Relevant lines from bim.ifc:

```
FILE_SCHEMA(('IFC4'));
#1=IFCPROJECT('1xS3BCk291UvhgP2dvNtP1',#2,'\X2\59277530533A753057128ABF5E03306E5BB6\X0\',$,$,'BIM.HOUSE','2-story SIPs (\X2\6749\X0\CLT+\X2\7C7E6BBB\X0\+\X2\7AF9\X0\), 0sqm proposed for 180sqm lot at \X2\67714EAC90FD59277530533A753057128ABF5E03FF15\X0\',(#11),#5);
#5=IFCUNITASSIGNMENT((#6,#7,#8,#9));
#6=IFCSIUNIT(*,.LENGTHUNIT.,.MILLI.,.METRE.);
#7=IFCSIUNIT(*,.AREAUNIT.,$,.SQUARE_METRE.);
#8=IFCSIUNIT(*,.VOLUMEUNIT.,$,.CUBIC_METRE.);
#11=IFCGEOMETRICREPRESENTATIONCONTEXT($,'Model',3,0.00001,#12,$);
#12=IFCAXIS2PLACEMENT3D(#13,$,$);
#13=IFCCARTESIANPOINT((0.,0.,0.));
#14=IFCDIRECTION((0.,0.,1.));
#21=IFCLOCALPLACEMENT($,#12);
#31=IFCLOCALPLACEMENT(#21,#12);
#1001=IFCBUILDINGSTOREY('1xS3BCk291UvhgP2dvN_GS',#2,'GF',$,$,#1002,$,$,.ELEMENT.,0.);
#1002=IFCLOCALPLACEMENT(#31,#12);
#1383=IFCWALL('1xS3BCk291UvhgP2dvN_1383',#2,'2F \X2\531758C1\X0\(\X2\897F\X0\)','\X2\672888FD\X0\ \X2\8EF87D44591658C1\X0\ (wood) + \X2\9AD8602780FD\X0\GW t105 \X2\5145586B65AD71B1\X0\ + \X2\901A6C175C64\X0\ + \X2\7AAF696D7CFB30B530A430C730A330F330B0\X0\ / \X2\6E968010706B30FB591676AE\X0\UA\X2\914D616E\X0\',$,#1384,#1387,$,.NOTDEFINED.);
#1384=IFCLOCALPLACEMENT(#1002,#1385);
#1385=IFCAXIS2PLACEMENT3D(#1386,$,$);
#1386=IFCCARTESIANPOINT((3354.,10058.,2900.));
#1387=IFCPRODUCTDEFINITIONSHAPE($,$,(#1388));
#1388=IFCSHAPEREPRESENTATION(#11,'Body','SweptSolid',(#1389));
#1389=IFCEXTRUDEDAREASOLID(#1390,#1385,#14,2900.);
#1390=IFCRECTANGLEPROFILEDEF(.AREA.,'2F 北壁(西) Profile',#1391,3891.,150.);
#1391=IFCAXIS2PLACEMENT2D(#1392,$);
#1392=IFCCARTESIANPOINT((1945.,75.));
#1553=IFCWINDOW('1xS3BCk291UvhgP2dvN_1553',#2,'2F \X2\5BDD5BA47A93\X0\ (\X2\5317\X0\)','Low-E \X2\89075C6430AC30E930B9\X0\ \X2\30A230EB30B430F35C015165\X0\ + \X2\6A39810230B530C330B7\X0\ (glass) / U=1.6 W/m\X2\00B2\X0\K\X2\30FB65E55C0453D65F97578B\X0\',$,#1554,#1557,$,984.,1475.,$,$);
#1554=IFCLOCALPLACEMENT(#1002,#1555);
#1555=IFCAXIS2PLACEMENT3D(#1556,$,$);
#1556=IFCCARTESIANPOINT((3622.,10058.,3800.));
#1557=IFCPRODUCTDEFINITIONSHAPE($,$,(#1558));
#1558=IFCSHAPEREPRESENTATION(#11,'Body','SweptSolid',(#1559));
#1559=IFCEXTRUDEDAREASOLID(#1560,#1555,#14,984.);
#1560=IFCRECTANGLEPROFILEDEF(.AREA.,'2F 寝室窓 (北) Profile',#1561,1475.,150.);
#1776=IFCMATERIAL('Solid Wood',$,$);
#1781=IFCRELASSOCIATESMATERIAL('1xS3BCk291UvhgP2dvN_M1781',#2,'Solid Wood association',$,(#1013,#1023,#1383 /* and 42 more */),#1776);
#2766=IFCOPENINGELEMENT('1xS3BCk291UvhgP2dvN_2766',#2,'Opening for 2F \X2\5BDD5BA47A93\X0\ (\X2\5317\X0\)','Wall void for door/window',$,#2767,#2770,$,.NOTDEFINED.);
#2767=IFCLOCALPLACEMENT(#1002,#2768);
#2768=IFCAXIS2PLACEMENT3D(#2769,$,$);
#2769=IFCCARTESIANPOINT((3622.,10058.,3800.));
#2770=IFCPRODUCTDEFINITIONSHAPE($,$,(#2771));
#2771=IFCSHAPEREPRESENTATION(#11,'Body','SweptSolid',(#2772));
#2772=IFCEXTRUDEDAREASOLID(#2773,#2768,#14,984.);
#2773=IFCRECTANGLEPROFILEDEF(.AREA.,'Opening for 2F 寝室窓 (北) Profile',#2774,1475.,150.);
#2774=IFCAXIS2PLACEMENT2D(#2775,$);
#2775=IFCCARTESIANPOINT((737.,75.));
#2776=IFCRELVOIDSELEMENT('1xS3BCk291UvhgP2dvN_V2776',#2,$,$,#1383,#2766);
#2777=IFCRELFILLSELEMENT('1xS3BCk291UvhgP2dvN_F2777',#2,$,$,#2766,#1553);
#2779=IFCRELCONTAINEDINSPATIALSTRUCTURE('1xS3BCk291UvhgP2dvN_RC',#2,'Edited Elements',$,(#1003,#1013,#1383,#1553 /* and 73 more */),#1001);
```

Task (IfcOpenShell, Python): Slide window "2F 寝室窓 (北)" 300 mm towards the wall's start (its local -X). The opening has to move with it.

```python
import ifcopenshell
import ifcopenshell.api.geometry
import ifcopenshell.util.placement

model = ifcopenshell.open("bim.ifc")

window = model.by_id(1553)
opening = window.FillsVoids[0].RelatingOpeningElement
wall = opening.VoidsElements[0].RelatingBuildingElement

wall_matrix = ifcopenshell.util.placement.get_local_placement(wall.ObjectPlacement)
shift = wall_matrix[:3, 0] * -300.0
before = ifcopenshell.util.placement.get_local_placement(window.ObjectPlacement)[:3, 3].copy()

# The window is not placed relative to its opening, so move both.
for product in (opening, window):
    matrix = ifcopenshell.util.placement.get_local_placement(product.ObjectPlacement)
    matrix[:3, 3] += shift
    ifcopenshell.api.geometry.edit_object_placement(model, product=product, matrix=matrix, is_si=False)

after = ifcopenshell.util.placement.get_local_placement(window.ObjectPlacement)[:3, 3]
print("window moved by", (after - before).round(3) + 0.0)

model.write("bim-out.ifc")
```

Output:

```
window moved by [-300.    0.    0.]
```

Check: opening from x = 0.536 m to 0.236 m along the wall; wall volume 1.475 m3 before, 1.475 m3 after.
